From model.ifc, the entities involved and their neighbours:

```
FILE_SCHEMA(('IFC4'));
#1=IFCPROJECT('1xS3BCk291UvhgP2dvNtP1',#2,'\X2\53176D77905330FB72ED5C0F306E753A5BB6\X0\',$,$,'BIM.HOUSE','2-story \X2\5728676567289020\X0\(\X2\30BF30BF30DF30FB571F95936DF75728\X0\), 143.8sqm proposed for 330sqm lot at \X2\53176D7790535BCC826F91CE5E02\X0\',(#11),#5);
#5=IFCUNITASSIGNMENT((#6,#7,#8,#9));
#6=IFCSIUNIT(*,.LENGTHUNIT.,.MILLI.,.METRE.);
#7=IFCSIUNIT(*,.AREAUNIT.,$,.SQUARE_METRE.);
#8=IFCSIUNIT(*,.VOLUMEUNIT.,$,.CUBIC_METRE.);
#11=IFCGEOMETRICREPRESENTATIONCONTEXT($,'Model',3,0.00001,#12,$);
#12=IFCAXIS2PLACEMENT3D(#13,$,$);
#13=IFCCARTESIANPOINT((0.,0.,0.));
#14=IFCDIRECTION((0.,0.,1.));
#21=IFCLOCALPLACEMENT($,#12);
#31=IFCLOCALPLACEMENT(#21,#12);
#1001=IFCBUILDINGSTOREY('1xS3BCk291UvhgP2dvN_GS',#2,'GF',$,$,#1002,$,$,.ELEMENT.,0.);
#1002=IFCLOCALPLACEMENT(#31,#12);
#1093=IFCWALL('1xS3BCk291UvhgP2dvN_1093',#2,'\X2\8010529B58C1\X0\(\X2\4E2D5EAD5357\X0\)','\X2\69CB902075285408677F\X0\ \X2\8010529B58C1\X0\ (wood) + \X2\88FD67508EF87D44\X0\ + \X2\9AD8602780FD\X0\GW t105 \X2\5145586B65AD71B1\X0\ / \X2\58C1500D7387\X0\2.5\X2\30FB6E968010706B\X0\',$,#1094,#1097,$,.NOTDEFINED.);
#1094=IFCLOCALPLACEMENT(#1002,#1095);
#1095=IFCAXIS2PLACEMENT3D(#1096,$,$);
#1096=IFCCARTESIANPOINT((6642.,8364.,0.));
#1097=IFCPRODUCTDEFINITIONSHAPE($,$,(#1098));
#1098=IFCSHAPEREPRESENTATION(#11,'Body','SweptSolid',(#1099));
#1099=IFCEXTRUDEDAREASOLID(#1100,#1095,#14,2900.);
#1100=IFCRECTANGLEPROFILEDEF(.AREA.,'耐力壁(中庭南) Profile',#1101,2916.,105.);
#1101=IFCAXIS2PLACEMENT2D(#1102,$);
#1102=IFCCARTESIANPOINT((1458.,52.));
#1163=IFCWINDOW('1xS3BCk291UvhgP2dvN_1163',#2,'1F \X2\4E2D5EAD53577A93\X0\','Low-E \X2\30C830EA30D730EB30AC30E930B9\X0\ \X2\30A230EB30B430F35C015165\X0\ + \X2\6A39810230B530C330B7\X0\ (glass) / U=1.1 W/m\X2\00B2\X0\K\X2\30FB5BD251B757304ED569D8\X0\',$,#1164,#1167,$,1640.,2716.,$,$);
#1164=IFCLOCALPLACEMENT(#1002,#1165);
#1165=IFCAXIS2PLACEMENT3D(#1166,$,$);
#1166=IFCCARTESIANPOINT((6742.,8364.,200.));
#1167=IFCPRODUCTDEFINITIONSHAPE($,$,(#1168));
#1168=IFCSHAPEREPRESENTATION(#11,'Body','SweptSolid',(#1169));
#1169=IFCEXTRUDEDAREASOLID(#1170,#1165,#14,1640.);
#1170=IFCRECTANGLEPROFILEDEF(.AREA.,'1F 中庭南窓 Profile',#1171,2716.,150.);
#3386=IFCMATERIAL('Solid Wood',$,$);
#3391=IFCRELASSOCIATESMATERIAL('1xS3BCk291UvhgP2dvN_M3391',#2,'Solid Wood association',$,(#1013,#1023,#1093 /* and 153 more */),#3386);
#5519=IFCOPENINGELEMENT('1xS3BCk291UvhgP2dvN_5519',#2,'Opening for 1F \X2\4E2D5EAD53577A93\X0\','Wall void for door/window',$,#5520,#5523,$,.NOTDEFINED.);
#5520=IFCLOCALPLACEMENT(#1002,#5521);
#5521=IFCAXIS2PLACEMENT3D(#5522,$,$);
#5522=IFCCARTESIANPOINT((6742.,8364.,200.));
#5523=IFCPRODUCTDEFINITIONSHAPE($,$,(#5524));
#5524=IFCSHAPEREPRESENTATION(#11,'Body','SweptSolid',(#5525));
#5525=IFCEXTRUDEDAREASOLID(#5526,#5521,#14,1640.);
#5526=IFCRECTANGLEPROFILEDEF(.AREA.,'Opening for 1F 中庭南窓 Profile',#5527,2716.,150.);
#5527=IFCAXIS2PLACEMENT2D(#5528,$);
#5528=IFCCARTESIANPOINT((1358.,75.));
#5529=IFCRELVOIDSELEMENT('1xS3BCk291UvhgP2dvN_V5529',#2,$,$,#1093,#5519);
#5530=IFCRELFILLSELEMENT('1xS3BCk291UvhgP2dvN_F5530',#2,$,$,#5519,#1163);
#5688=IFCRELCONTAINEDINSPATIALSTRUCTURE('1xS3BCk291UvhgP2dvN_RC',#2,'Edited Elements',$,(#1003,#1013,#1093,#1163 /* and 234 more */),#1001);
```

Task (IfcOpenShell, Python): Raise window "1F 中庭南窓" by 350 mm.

```python
import numpy as np
import ifcopenshell
import ifcopenshell.api.geometry
import ifcopenshell.util.placement
import ifcopenshell.util.unit

model = ifcopenshell.open("model.ifc")
unit_scale = ifcopenshell.util.unit.calculate_unit_scale(model)

window = model.by_guid("1xS3BCk291UvhgP2dvN_1163")
opening = window.FillsVoids[0].RelatingOpeningElement
dz = 350.0

shift = np.array([0.0, 0.0, dz])
# The window is not placed relative to its opening, so move both.
for product in (opening, window):
    matrix = ifcopenshell.util.placement.get_local_placement(product.ObjectPlacement)
    matrix[:3, 3] += shift
    ifcopenshell.api.geometry.edit_object_placement(model, product=product, matrix=matrix, is_si=False)

print(f"moved by {dz * unit_scale:+.3f} m")

model.write("model-out.ifc")
```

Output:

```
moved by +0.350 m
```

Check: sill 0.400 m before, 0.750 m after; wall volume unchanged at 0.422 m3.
